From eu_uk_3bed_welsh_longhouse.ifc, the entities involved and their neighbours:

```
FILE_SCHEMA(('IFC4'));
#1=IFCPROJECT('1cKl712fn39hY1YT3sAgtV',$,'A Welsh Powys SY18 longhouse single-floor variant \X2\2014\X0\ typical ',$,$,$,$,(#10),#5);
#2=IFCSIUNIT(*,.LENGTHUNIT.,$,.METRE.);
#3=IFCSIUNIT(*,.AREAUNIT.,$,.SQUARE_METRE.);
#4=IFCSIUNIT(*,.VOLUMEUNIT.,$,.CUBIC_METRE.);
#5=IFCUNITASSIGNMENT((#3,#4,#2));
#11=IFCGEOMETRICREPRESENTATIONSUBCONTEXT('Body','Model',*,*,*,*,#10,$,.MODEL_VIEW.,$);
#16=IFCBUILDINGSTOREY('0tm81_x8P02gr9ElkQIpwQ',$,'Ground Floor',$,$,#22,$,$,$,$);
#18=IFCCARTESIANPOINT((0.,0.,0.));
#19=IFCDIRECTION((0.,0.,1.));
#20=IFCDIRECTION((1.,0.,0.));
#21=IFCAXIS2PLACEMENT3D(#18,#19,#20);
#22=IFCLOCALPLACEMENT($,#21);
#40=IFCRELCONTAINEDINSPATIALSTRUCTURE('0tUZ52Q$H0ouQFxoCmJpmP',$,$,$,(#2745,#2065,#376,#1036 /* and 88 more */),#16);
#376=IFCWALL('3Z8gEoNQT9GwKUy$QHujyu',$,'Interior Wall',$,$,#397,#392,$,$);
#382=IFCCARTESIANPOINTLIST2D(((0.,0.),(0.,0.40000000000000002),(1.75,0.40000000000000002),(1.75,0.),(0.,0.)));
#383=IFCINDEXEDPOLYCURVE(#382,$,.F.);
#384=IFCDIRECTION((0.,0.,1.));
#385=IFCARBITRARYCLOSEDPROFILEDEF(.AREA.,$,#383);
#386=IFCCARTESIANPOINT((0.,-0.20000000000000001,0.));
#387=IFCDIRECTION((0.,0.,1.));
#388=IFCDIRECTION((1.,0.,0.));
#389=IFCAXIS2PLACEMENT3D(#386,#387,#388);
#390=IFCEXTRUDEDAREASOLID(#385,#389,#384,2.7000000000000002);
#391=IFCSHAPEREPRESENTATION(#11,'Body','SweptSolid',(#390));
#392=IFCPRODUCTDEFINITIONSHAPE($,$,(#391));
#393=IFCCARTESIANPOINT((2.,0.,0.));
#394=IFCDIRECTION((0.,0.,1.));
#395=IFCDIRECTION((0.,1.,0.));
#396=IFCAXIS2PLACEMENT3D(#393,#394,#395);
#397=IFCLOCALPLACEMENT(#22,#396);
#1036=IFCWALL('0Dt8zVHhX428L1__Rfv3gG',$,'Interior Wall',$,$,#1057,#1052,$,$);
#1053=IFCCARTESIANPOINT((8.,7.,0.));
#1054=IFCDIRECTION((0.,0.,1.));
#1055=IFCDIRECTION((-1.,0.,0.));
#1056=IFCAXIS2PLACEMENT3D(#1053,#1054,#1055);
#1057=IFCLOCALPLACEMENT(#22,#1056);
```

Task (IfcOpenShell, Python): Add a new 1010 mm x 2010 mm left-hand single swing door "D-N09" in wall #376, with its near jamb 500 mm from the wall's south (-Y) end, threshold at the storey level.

```python
import numpy as np
import ifcopenshell
import ifcopenshell.api.feature
import ifcopenshell.api.geometry
import ifcopenshell.api.root
import ifcopenshell.api.spatial
import ifcopenshell.geom
import ifcopenshell.util.element
import ifcopenshell.util.placement
import ifcopenshell.util.representation
import ifcopenshell.util.shape
import ifcopenshell.util.unit

model = ifcopenshell.open("eu_uk_3bed_welsh_longhouse.ifc")
unit_scale = ifcopenshell.util.unit.calculate_unit_scale(model)
settings = ifcopenshell.geom.settings()


def volume(element):
    """Net volume in cubic metres, openings subtracted."""
    shape = ifcopenshell.geom.create_shape(settings, element)
    return ifcopenshell.util.shape.get_volume(shape.geometry)


wall = model.by_guid("3Z8gEoNQT9GwKUy$QHujyu")
storey = ifcopenshell.util.element.get_container(wall, ifc_class="IfcBuildingStorey")
context = ifcopenshell.util.representation.get_context(model, "Model", "Body", "MODEL_VIEW")
before = volume(wall)

width, height, from_end, sill = 1.01, 2.01, 0.5, 0.0  # metres

# The wall runs along its own X axis, and the end named is its -X end.
wall_shape = ifcopenshell.geom.create_shape(settings, wall)
x, y, z = ifcopenshell.util.shape.get_vertices(wall_shape.geometry).T
start = x.min() + from_end
face, thickness = float(y.min()), float(y.max() - y.min())
wall_matrix = ifcopenshell.util.placement.get_local_placement(wall.ObjectPlacement)
level = ifcopenshell.util.placement.get_local_placement(storey.ObjectPlacement)[2, 3]


def in_wall(x, y):
    """Placement at x, y metres in the wall's axes, at sill height."""
    matrix = wall_matrix.copy()
    matrix[:, 3] = wall_matrix @ np.array([x / unit_scale, y / unit_scale, 0.0, 1.0])
    matrix[2, 3] = level + sill / unit_scale
    return matrix


# Opening: a box that overshoots both wall faces by 50 mm.
opening = ifcopenshell.api.root.create_entity(model, ifc_class="IfcOpeningElement", predefined_type="OPENING")
box = ifcopenshell.api.geometry.add_wall_representation(
    model, context=context, length=width, height=height, thickness=thickness + 0.1
)
ifcopenshell.api.geometry.assign_representation(model, product=opening, representation=box)
ifcopenshell.api.geometry.edit_object_placement(model, product=opening, matrix=in_wall(start, face - 0.05), is_si=False)
ifcopenshell.api.feature.add_feature(model, feature=opening, element=wall)

door = ifcopenshell.api.root.create_entity(model, ifc_class="IfcDoor", name="D-N09", predefined_type="DOOR")
door.OverallWidth, door.OverallHeight = width / unit_scale, height / unit_scale
door.OperationType = "SINGLE_SWING_LEFT"
body = ifcopenshell.api.geometry.add_door_representation(
    model,
    context=context,
    overall_width=door.OverallWidth,
    overall_height=door.OverallHeight,
    operation_type="SINGLE_SWING_LEFT",
    lining_properties={"LiningDepth": thickness / unit_scale, "ThresholdDepth": thickness / unit_scale},
)
ifcopenshell.api.geometry.assign_representation(model, product=door, representation=body)
ifcopenshell.api.spatial.assign_container(model, products=[door], relating_structure=storey)
ifcopenshell.api.feature.add_filling(model, opening=opening, element=door)

# The lining spans the wall, so the door starts at the wall face.
ifcopenshell.api.geometry.edit_object_placement(model, product=door, matrix=in_wall(start, face), is_si=False)

after = volume(wall)

print(f"wall volume {before:.3f} -> {after:.3f} m3")

model.write("eu_uk_3bed_welsh_longhouse_rev.ifc")
```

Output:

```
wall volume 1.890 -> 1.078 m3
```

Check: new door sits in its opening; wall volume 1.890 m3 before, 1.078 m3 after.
